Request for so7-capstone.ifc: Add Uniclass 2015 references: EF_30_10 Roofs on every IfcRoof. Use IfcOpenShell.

First a look at what the model holds.

```python
import ifcopenshell

model = ifcopenshell.open("so7-capstone.ifc")
print(model.schema)
print("classifications:", [c.Name for c in model.by_type("IfcClassification")])
for ifc_class in ("IfcDoor", "IfcRoof", "IfcStair", "IfcWall", "IfcWindow"):
    print(ifc_class, len(model.by_type(ifc_class)))
```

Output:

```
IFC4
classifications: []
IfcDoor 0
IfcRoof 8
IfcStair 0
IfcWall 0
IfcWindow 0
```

```python
import ifcopenshell
import ifcopenshell.api.classification

model = ifcopenshell.open("so7-capstone.ifc")

system = ifcopenshell.api.classification.add_classification(model, classification="Uniclass 2015")

codes = {
    "IfcRoof": ("EF_30_10", "Roofs"),
}
for ifc_class, (code, name) in codes.items():
    products = model.by_type(ifc_class)
    ifcopenshell.api.classification.add_reference(
        model, products=products, classification=system, identification=code, name=name
    )
    print(code, len(products))

model.write("so7-capstone_edited.ifc")
```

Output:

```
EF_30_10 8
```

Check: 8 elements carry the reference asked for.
